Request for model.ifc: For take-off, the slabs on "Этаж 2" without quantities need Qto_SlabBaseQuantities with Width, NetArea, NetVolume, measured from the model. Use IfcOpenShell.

First a look at what the model holds.

```python
import ifcopenshell
import ifcopenshell.util.element
import ifcopenshell.util.unit

model = ifcopenshell.open("model.ifc")
print(model.schema)
for unit_type in ("LENGTHUNIT", "AREAUNIT", "VOLUMEUNIT"):
    print(unit_type, ifcopenshell.util.unit.calculate_unit_scale(model, unit_type))
storey = next(s for s in model.by_type("IfcBuildingStorey") if s.Name == "Этаж 2")
slabs = [e for e in ifcopenshell.util.element.get_decomposition(storey) if e.is_a("IfcSlab")]
for e in sorted(slabs, key=lambda e: e.id()):
    print(e.id(), e.is_a(), e.Name, list(ifcopenshell.util.element.get_psets(e, qtos_only=True)), sep=" | ")
```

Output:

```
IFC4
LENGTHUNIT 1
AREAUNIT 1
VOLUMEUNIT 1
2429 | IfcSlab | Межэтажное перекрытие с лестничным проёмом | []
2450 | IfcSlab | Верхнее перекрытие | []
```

```python
import ifcopenshell
import ifcopenshell.api.pset
import ifcopenshell.geom
import ifcopenshell.util.element
import ifcopenshell.util.shape
import ifcopenshell.util.unit

model = ifcopenshell.open("model.ifc")
unit_scale = ifcopenshell.util.unit.calculate_unit_scale(model)
area_scale = ifcopenshell.util.unit.calculate_unit_scale(model, "AREAUNIT")
volume_scale = ifcopenshell.util.unit.calculate_unit_scale(model, "VOLUMEUNIT")
settings = ifcopenshell.geom.settings()

storey = next(s for s in model.by_type("IfcBuildingStorey") if s.Name == "Этаж 2")
slabs = [e for e in ifcopenshell.util.element.get_decomposition(storey) if e.is_a("IfcSlab")]

for e in sorted(slabs, key=lambda e: e.id()):
    if ifcopenshell.util.element.get_psets(e, qtos_only=True, should_inherit=False):
        continue
    # Geometry comes back in metres, in the element's own axes.
    shape = ifcopenshell.geom.create_shape(settings, e)
    values = {
        "Width": ifcopenshell.util.shape.get_z(shape.geometry) / unit_scale,
        "NetArea": ifcopenshell.util.shape.get_footprint_area(shape.geometry) / area_scale,
        "NetVolume": ifcopenshell.util.shape.get_volume(shape.geometry) / volume_scale,
    }
    qto = ifcopenshell.api.pset.add_qto(model, product=e, name="Qto_SlabBaseQuantities")
    ifcopenshell.api.pset.edit_qto(model, qto=qto, properties=values)
    print(e.id(), {k: round(v, 3) for k, v in values.items()})

model.write("model_edited.ifc")
```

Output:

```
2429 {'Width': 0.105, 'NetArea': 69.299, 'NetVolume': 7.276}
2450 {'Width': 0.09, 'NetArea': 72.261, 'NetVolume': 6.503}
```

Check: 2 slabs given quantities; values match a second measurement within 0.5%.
